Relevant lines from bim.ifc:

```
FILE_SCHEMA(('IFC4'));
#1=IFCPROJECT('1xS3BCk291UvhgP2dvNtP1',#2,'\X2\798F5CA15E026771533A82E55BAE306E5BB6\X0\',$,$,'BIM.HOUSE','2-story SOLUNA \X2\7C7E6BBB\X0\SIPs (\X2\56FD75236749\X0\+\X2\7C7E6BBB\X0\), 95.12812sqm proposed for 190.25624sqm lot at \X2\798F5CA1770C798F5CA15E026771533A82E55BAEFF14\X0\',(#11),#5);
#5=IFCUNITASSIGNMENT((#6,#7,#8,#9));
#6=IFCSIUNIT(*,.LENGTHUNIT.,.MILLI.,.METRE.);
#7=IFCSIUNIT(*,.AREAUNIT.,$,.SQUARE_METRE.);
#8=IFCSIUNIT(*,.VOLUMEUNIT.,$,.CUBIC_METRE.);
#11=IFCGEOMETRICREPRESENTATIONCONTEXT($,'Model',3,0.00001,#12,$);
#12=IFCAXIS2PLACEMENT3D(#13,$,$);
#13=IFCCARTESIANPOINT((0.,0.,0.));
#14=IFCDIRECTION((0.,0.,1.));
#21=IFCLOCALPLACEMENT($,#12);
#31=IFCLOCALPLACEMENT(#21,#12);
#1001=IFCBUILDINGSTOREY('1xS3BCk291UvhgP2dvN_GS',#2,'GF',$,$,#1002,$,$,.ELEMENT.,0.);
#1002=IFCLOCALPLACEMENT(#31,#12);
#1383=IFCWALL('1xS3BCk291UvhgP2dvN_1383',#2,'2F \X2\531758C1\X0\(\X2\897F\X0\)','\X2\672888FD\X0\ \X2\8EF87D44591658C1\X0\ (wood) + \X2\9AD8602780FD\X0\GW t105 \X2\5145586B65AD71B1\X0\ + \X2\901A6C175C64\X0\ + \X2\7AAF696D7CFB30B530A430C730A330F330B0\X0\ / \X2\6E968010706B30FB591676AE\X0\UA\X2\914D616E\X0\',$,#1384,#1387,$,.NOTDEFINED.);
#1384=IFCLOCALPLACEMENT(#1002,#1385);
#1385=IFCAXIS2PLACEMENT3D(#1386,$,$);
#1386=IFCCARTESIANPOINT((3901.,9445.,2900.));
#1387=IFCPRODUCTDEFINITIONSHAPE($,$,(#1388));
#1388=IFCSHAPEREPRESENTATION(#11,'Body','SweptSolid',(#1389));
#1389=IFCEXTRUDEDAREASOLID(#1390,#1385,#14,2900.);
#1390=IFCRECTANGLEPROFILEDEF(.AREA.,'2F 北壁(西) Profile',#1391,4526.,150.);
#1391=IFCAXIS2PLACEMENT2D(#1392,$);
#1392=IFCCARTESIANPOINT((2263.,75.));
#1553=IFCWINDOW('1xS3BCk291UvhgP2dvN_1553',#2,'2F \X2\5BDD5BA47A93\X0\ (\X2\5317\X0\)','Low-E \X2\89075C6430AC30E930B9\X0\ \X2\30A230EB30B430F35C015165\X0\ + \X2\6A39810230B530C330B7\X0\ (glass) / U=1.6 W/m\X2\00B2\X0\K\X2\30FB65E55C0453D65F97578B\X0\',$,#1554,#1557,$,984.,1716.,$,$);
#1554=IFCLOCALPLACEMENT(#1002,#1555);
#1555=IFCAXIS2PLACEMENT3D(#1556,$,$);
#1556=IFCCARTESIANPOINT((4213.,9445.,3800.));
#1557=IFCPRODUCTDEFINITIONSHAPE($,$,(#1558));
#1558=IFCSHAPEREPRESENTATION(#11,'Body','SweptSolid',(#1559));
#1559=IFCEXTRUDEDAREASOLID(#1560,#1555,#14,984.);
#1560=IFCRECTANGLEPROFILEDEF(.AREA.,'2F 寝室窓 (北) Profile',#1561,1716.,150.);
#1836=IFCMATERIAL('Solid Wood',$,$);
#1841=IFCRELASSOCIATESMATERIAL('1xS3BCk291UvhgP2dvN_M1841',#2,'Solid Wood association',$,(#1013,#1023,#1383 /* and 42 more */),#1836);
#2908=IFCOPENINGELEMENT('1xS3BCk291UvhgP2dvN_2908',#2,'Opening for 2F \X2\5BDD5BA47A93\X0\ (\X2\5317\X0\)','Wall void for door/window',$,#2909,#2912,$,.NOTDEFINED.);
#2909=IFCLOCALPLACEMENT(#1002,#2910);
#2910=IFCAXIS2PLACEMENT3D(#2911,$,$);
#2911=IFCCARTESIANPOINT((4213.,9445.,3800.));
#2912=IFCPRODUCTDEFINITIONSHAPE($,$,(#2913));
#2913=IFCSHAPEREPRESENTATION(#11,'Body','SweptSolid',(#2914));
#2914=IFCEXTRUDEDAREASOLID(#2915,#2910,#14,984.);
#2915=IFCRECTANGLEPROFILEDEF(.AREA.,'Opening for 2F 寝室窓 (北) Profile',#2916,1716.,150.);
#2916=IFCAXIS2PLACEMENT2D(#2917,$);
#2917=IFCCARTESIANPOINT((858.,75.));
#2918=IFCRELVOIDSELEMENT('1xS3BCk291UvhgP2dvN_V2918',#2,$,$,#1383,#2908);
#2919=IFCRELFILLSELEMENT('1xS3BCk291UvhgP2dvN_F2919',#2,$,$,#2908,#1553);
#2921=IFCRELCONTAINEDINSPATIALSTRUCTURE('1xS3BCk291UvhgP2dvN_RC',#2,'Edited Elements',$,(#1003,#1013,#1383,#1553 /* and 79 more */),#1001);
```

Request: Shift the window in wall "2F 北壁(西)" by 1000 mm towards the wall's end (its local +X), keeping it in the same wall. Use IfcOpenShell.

```python
import ifcopenshell
import ifcopenshell.api.geometry
import ifcopenshell.util.placement

model = ifcopenshell.open("bim.ifc")

window = model.by_guid("1xS3BCk291UvhgP2dvN_1553")
opening = window.FillsVoids[0].RelatingOpeningElement
wall = opening.VoidsElements[0].RelatingBuildingElement

wall_matrix = ifcopenshell.util.placement.get_local_placement(wall.ObjectPlacement)
shift = wall_matrix[:3, 0] * 1000.0
before = ifcopenshell.util.placement.get_local_placement(window.ObjectPlacement)[:3, 3].copy()

# The window is not placed relative to its opening, so move both.
for product in (opening, window):
    matrix = ifcopenshell.util.placement.get_local_placement(product.ObjectPlacement)
    matrix[:3, 3] += shift
    ifcopenshell.api.geometry.edit_object_placement(model, product=product, matrix=matrix, is_si=False)

after = ifcopenshell.util.placement.get_local_placement(window.ObjectPlacement)[:3, 3]
print("window moved by", (after - before).round(3) + 0.0)

model.write("bim-out.ifc")
```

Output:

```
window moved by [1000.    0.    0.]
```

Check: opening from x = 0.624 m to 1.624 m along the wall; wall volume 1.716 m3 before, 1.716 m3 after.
